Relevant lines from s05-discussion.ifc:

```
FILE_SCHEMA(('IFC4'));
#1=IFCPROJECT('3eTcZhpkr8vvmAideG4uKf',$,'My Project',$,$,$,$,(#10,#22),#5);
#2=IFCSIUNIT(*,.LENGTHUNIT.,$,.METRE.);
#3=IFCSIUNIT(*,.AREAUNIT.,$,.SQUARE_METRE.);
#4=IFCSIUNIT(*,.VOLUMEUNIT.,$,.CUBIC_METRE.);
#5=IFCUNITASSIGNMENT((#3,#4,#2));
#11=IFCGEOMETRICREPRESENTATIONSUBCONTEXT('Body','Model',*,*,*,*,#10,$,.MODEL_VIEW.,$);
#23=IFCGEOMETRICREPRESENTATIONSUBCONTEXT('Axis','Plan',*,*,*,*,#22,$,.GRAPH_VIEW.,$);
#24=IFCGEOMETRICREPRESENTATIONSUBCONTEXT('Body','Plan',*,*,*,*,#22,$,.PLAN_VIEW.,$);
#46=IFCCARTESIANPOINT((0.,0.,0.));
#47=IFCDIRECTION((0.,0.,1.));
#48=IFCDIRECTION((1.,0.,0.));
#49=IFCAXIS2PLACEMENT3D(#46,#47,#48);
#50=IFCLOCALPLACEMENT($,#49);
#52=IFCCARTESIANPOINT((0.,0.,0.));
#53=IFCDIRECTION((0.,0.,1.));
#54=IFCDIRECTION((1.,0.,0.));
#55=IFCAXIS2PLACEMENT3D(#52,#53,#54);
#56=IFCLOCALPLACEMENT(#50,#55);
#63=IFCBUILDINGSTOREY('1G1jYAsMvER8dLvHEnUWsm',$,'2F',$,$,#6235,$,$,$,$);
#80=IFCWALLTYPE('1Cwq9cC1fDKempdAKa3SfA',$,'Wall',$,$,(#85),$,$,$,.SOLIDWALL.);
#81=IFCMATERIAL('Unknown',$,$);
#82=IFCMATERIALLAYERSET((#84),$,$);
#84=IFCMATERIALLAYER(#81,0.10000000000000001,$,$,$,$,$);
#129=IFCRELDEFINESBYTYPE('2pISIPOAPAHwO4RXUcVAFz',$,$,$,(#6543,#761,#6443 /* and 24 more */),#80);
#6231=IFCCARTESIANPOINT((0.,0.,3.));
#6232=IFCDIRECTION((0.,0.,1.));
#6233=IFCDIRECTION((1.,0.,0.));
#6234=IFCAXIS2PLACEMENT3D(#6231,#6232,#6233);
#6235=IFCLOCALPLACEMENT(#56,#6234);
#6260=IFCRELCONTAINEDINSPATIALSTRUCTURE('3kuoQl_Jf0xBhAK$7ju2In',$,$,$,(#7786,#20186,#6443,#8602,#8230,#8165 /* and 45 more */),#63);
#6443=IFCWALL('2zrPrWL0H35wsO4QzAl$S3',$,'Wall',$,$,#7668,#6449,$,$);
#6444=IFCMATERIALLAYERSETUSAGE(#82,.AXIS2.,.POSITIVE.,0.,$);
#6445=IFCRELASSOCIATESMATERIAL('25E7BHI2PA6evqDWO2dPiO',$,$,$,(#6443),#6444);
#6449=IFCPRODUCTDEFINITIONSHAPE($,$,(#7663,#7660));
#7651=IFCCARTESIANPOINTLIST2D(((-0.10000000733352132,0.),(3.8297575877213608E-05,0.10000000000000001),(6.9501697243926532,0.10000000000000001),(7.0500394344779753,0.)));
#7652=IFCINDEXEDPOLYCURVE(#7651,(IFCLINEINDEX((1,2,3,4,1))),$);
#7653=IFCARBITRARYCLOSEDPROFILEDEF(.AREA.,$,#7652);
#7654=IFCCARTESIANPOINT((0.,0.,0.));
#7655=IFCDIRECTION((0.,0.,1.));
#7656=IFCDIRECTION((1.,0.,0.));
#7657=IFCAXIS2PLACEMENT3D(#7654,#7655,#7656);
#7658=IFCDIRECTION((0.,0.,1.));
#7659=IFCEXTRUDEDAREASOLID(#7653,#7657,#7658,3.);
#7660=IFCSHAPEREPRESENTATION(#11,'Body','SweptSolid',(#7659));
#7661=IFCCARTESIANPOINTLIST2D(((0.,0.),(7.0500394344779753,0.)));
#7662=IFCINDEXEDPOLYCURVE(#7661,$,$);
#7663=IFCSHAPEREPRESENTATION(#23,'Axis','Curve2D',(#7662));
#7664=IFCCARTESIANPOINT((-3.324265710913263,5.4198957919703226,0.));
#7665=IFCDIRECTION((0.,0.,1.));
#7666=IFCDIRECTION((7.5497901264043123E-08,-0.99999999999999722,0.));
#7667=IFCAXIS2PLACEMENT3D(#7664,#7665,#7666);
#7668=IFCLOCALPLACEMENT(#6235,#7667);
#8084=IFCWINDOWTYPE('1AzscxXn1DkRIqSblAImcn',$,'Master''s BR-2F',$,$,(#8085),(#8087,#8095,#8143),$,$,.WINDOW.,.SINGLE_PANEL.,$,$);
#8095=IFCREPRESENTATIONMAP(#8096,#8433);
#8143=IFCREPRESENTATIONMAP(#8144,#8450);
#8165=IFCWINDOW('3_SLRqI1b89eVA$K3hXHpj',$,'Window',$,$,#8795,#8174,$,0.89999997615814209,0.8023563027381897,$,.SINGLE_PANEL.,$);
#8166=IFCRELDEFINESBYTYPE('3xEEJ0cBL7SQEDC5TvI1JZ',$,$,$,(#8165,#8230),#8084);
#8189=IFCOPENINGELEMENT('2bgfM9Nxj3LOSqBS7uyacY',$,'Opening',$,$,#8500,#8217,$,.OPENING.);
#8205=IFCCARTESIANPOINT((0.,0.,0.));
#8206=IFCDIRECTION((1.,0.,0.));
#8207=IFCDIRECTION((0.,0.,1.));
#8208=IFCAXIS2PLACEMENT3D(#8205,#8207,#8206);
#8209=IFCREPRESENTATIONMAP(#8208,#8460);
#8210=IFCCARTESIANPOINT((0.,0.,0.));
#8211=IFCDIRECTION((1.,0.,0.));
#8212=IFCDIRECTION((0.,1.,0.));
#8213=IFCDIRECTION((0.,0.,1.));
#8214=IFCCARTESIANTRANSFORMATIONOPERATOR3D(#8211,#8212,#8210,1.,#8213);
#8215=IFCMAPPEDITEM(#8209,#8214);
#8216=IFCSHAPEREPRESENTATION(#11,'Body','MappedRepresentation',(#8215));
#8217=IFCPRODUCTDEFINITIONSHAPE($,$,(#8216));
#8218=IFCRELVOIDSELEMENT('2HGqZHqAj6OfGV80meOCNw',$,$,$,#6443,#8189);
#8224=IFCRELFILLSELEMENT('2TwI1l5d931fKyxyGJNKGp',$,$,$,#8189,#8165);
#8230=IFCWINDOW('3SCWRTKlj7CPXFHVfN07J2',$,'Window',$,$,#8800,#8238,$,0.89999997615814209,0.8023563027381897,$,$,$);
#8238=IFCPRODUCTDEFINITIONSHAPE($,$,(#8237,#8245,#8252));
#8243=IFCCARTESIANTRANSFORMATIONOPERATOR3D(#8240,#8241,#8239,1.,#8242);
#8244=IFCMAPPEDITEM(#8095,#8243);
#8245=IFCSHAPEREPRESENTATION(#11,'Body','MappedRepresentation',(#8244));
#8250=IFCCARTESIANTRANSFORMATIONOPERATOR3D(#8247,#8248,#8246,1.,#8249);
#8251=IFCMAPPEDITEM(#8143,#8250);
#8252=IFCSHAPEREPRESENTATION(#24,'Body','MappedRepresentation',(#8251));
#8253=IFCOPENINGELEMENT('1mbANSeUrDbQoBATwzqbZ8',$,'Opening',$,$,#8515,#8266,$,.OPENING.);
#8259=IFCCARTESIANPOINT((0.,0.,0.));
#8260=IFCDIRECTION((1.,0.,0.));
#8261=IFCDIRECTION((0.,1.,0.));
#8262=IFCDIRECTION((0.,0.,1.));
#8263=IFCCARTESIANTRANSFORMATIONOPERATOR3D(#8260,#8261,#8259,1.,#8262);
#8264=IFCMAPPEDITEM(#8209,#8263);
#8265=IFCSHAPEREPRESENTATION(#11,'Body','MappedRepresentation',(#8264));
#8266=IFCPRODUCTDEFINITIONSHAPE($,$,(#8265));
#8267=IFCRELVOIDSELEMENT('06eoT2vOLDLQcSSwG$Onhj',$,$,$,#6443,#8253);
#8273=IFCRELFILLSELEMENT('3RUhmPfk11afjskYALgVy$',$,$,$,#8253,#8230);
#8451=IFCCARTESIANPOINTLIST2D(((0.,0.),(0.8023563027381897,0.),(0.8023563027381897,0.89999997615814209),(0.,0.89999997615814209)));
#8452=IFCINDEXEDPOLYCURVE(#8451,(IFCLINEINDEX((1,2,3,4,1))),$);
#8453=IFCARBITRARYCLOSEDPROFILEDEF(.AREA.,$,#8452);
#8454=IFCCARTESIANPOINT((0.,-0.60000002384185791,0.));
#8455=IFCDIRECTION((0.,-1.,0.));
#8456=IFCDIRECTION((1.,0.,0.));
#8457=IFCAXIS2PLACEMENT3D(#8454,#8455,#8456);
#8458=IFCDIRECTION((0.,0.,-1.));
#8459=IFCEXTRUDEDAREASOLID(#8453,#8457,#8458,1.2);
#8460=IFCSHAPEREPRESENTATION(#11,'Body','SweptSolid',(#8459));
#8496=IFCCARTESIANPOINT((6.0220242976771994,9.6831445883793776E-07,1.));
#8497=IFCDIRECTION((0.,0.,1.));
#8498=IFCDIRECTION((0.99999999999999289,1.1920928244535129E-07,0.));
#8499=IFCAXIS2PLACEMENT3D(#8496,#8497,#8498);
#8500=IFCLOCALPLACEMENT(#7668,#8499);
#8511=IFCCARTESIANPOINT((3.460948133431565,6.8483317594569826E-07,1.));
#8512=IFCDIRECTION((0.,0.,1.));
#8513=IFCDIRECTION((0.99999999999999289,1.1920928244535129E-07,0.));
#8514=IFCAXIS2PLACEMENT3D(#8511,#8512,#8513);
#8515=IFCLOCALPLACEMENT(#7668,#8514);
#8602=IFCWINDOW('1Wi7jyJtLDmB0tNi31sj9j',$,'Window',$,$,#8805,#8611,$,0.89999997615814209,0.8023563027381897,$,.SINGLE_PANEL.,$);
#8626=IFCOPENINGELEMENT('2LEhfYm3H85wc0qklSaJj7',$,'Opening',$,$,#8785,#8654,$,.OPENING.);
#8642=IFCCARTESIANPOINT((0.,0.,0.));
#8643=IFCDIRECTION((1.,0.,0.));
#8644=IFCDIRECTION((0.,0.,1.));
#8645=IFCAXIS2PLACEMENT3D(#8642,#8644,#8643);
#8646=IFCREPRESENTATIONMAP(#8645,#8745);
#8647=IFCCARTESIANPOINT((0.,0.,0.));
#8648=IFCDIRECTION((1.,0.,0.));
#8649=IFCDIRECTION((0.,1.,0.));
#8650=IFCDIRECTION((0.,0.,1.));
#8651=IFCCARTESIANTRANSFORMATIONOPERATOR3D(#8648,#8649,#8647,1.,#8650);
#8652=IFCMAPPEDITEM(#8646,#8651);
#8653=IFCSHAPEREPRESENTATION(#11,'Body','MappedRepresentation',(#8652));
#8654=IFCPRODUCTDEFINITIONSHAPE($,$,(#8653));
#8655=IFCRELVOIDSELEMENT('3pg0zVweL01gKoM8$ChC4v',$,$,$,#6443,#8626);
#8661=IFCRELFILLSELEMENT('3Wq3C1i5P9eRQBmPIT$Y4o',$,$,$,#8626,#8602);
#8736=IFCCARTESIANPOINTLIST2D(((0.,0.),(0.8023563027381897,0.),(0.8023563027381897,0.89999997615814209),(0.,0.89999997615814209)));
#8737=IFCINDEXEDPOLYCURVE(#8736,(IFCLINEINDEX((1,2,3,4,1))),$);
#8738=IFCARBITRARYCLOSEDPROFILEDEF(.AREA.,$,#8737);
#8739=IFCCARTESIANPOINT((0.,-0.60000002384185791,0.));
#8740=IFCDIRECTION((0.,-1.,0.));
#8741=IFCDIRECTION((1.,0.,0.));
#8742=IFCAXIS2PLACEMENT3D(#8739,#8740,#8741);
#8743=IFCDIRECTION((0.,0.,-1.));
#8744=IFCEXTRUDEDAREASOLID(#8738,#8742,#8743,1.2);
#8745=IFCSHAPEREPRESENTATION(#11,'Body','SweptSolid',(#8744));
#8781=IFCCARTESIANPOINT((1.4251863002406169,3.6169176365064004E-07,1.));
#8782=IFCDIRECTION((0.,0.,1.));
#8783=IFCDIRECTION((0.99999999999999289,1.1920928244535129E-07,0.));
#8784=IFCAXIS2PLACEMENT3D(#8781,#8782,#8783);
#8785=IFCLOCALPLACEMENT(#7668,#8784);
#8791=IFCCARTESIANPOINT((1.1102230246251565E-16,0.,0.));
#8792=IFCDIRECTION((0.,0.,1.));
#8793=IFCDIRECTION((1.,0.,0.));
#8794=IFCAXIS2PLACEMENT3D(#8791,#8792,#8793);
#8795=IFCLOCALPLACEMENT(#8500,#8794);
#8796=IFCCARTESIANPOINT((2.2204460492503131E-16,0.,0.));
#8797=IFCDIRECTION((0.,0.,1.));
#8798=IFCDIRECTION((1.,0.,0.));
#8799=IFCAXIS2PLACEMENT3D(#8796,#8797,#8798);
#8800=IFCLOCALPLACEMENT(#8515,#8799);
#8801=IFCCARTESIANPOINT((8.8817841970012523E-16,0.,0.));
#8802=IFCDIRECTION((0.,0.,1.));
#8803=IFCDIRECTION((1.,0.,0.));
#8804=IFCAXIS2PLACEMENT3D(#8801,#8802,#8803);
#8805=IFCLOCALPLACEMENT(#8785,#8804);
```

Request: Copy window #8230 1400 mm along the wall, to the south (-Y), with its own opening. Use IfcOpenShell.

```python
import ifcopenshell
import ifcopenshell.api.feature
import ifcopenshell.api.geometry
import ifcopenshell.api.root
import ifcopenshell.geom
import ifcopenshell.util.element
import ifcopenshell.util.placement
import ifcopenshell.util.shape
import ifcopenshell.util.unit

model = ifcopenshell.open("s05-discussion.ifc")
unit_scale = ifcopenshell.util.unit.calculate_unit_scale(model)
settings = ifcopenshell.geom.settings()


def volume(element):
    """Net volume in cubic metres, openings subtracted."""
    shape = ifcopenshell.geom.create_shape(settings, element)
    return ifcopenshell.util.shape.get_volume(shape.geometry)


window = model.by_guid("3SCWRTKlj7CPXFHVfN07J2")
opening = window.FillsVoids[0].RelatingOpeningElement
wall = opening.VoidsElements[0].RelatingBuildingElement
before = volume(wall)
shift = ifcopenshell.util.placement.get_local_placement(wall.ObjectPlacement)[:3, 0] * 1.4 / unit_scale

# copy_class copies the void relationship, type, container and properties, but no geometry.
new_opening = ifcopenshell.api.root.copy_class(model, product=opening)
new_opening.Representation = ifcopenshell.util.element.copy_deep(
    model, opening.Representation, exclude=["IfcGeometricRepresentationContext", "IfcRepresentationMap"]
)
new_window = ifcopenshell.api.root.copy_class(model, product=window)
new_window.Representation = ifcopenshell.util.element.copy_deep(
    model, window.Representation, exclude=["IfcGeometricRepresentationContext", "IfcRepresentationMap"]
)
ifcopenshell.api.feature.add_filling(model, opening=new_opening, element=new_window)

for old, new in ((opening, new_opening), (window, new_window)):
    matrix = ifcopenshell.util.placement.get_local_placement(old.ObjectPlacement)
    matrix[:3, 3] += shift
    ifcopenshell.api.geometry.edit_object_placement(model, product=new, matrix=matrix, is_si=False)

after = volume(wall)

print(f"wall volume {before:.3f} -> {after:.3f} m3")

model.write("s05-discussion_updated.ifc")
```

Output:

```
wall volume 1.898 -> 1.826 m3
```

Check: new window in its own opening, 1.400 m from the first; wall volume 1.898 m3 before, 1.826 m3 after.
